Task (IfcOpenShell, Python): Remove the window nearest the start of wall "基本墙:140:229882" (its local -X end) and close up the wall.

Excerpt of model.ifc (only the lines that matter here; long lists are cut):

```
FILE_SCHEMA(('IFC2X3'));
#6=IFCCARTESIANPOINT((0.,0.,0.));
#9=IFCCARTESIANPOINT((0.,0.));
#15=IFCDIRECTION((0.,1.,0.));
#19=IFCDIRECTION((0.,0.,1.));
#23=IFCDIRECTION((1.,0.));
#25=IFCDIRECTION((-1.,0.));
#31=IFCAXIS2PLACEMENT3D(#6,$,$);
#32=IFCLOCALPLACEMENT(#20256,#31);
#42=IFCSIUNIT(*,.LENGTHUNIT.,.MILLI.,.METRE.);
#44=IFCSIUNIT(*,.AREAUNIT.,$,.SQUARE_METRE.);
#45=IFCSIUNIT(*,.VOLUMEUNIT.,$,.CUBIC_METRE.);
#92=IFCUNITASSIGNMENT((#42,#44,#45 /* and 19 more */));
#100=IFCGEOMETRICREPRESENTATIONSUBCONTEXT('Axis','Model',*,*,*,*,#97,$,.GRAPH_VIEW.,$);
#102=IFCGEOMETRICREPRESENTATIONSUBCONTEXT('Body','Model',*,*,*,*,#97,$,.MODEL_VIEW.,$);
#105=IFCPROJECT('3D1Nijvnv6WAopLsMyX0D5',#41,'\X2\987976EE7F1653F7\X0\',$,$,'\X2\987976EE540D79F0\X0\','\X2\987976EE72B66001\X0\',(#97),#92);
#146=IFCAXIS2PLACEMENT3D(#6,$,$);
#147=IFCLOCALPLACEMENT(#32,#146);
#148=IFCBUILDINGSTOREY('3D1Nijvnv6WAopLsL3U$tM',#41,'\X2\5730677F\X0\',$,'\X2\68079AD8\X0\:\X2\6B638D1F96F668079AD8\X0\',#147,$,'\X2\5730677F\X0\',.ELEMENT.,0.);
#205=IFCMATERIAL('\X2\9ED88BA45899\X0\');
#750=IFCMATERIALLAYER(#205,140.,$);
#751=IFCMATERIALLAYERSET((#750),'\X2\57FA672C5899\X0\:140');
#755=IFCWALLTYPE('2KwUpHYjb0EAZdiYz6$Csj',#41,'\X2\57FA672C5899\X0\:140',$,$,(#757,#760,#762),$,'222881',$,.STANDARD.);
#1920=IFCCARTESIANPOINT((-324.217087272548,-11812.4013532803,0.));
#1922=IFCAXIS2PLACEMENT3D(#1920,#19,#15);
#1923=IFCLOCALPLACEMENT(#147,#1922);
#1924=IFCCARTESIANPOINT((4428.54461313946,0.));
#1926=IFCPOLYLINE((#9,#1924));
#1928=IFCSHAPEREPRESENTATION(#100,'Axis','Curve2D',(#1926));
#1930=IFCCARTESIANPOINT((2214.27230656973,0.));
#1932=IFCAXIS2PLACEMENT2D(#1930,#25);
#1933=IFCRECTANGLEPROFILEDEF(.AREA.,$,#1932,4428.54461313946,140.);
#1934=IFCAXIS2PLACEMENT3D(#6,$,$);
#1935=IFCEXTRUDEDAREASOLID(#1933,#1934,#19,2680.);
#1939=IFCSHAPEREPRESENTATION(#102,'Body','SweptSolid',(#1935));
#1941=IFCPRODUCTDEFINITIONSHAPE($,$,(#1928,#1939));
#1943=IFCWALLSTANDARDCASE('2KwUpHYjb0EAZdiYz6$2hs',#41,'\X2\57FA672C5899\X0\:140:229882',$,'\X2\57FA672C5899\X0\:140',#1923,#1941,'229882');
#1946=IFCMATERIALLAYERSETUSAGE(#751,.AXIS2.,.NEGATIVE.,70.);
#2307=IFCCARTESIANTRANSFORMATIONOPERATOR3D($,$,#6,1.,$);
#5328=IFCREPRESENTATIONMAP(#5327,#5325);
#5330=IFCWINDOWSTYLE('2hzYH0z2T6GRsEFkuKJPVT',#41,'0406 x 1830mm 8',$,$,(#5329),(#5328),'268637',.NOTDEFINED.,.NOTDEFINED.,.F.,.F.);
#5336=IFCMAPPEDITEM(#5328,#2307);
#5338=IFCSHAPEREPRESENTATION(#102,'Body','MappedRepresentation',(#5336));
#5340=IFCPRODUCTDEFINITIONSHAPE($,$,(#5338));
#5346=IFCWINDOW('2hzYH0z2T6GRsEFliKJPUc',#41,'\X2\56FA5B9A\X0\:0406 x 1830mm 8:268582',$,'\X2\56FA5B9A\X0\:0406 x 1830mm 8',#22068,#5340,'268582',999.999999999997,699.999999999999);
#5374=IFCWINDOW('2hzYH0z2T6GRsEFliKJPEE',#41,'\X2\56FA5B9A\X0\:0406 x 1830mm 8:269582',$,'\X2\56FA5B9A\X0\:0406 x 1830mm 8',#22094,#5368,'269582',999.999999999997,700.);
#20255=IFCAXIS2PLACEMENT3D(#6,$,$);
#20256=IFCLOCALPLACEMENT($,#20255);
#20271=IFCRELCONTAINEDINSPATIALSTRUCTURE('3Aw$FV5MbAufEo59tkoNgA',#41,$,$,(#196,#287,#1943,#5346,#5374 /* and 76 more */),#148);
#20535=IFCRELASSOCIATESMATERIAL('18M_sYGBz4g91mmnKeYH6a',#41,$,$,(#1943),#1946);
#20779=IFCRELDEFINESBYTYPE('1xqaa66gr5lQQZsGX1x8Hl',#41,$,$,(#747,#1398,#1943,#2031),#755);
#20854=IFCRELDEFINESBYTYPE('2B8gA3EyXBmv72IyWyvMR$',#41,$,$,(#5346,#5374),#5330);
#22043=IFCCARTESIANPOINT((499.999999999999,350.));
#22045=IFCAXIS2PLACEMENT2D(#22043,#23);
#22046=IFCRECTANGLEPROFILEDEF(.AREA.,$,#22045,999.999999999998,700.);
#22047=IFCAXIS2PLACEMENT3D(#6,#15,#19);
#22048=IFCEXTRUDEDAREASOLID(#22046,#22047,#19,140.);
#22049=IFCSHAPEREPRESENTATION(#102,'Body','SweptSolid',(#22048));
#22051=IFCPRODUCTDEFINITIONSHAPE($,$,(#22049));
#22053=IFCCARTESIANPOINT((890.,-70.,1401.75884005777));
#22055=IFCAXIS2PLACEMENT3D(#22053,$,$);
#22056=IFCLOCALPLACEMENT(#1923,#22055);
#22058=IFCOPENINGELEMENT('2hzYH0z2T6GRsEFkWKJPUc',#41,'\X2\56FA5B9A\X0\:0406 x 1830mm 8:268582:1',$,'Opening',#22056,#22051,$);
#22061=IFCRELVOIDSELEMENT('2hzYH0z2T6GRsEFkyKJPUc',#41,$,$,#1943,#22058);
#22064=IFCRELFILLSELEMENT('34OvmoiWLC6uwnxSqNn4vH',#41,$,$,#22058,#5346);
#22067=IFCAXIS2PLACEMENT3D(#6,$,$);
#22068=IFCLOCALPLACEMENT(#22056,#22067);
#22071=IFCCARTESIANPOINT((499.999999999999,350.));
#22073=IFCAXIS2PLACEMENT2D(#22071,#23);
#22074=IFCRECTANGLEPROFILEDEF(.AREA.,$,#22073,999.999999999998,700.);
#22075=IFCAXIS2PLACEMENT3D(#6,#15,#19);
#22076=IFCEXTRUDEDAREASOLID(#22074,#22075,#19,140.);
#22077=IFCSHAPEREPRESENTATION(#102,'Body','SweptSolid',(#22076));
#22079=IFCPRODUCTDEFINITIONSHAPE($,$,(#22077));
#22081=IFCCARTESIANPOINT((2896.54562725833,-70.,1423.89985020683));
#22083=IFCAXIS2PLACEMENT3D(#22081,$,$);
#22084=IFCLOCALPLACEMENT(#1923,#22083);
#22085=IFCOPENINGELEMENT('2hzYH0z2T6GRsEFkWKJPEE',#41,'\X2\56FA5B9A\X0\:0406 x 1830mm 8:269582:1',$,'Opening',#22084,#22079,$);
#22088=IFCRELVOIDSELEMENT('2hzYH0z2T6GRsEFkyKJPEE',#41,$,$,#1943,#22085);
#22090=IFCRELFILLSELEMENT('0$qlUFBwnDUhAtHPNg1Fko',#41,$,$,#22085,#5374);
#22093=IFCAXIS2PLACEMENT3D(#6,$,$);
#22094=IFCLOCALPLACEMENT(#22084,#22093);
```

```python
import ifcopenshell
import ifcopenshell.api.feature
import ifcopenshell.api.root
import ifcopenshell.geom
import ifcopenshell.util.shape

model = ifcopenshell.open("model.ifc")
settings = ifcopenshell.geom.settings()


def volume(element):
    """Net volume in cubic metres, openings subtracted."""
    shape = ifcopenshell.geom.create_shape(settings, element)
    return ifcopenshell.util.shape.get_volume(shape.geometry)


window = model.by_guid("2hzYH0z2T6GRsEFliKJPUc")
opening = window.FillsVoids[0].RelatingOpeningElement
wall = opening.VoidsElements[0].RelatingBuildingElement
before = volume(wall)

ifcopenshell.api.root.remove_product(model, product=window)
ifcopenshell.api.feature.remove_feature(model, feature=opening)

after = volume(wall)

print(f"wall volume {before:.3f} -> {after:.3f} m3")

model.write("model_edited.ifc")
```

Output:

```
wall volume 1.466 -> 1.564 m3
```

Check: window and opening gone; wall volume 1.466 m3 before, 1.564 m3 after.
